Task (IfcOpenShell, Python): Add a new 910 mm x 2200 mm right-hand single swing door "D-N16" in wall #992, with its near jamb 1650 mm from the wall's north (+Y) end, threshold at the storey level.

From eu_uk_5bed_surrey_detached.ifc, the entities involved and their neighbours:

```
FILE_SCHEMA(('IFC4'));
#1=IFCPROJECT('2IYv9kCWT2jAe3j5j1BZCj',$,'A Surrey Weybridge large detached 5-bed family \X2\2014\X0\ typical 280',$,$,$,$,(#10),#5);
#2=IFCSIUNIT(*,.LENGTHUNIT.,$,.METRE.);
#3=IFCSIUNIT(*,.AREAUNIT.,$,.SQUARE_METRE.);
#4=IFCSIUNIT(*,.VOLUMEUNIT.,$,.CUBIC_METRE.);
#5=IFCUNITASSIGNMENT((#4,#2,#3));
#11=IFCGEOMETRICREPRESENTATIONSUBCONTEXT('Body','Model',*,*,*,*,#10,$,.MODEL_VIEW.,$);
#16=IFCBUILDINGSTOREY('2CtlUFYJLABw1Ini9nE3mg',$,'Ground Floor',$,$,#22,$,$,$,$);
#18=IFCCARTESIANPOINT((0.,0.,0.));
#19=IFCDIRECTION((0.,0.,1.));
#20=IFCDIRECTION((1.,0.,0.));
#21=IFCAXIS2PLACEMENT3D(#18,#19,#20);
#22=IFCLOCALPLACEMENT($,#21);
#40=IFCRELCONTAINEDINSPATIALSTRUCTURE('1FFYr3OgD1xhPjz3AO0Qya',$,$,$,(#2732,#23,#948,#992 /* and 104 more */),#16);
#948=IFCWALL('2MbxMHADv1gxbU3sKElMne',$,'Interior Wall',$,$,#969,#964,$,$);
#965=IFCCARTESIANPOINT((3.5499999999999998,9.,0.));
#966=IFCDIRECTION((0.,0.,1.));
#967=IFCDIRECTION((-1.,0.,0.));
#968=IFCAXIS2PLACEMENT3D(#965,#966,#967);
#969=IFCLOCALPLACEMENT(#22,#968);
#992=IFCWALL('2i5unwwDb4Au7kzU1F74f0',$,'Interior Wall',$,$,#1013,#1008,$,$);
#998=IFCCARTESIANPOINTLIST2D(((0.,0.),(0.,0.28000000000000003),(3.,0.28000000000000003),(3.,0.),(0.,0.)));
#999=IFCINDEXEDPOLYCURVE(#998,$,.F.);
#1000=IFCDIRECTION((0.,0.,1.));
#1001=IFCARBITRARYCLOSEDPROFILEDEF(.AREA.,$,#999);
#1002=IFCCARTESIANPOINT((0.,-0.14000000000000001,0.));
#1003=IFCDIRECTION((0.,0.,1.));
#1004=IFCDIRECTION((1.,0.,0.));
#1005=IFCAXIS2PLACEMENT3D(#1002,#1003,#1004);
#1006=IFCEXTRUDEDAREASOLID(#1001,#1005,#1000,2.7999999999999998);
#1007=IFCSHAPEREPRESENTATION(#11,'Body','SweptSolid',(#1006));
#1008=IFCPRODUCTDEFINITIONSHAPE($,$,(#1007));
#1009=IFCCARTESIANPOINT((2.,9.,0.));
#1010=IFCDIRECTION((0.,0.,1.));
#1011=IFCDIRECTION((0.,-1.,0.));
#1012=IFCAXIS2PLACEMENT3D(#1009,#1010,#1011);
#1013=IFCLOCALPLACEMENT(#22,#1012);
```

```python
import numpy as np
import ifcopenshell
import ifcopenshell.api.feature
import ifcopenshell.api.geometry
import ifcopenshell.api.root
import ifcopenshell.api.spatial
import ifcopenshell.geom
import ifcopenshell.util.element
import ifcopenshell.util.placement
import ifcopenshell.util.representation
import ifcopenshell.util.shape
import ifcopenshell.util.unit

model = ifcopenshell.open("eu_uk_5bed_surrey_detached.ifc")
unit_scale = ifcopenshell.util.unit.calculate_unit_scale(model)
settings = ifcopenshell.geom.settings()


def volume(element):
    """Net volume in cubic metres, openings subtracted."""
    shape = ifcopenshell.geom.create_shape(settings, element)
    return ifcopenshell.util.shape.get_volume(shape.geometry)


wall = model.by_guid("2i5unwwDb4Au7kzU1F74f0")
storey = ifcopenshell.util.element.get_container(wall, ifc_class="IfcBuildingStorey")
context = ifcopenshell.util.representation.get_context(model, "Model", "Body", "MODEL_VIEW")
before = volume(wall)

width, height, from_end, sill = 0.91, 2.2, 1.65, 0.0  # metres

# The wall runs along its own X axis, and the end named is its -X end.
wall_shape = ifcopenshell.geom.create_shape(settings, wall)
x, y, z = ifcopenshell.util.shape.get_vertices(wall_shape.geometry).T
start = x.min() + from_end
face, thickness = float(y.min()), float(y.max() - y.min())
wall_matrix = ifcopenshell.util.placement.get_local_placement(wall.ObjectPlacement)
level = ifcopenshell.util.placement.get_local_placement(storey.ObjectPlacement)[2, 3]


def in_wall(x, y):
    """Placement at x, y metres in the wall's axes, at sill height."""
    matrix = wall_matrix.copy()
    matrix[:, 3] = wall_matrix @ np.array([x / unit_scale, y / unit_scale, 0.0, 1.0])
    matrix[2, 3] = level + sill / unit_scale
    return matrix


# Opening: a box that overshoots both wall faces by 50 mm.
opening = ifcopenshell.api.root.create_entity(model, ifc_class="IfcOpeningElement", predefined_type="OPENING")
box = ifcopenshell.api.geometry.add_wall_representation(
    model, context=context, length=width, height=height, thickness=thickness + 0.1
)
ifcopenshell.api.geometry.assign_representation(model, product=opening, representation=box)
ifcopenshell.api.geometry.edit_object_placement(model, product=opening, matrix=in_wall(start, face - 0.05), is_si=False)
ifcopenshell.api.feature.add_feature(model, feature=opening, element=wall)

door = ifcopenshell.api.root.create_entity(model, ifc_class="IfcDoor", name="D-N16", predefined_type="DOOR")
door.OverallWidth, door.OverallHeight = width / unit_scale, height / unit_scale
door.OperationType = "SINGLE_SWING_RIGHT"
body = ifcopenshell.api.geometry.add_door_representation(
    model,
    context=context,
    overall_width=door.OverallWidth,
    overall_height=door.OverallHeight,
    operation_type="SINGLE_SWING_RIGHT",
    lining_properties={"LiningDepth": thickness / unit_scale, "ThresholdDepth": thickness / unit_scale},
)
ifcopenshell.api.geometry.assign_representation(model, product=door, representation=body)
ifcopenshell.api.spatial.assign_container(model, products=[door], relating_structure=storey)
ifcopenshell.api.feature.add_filling(model, opening=opening, element=door)

# The lining spans the wall, so the door starts at the wall face.
ifcopenshell.api.geometry.edit_object_placement(model, product=door, matrix=in_wall(start, face), is_si=False)

after = volume(wall)

print(f"wall volume {before:.3f} -> {after:.3f} m3")

model.write("eu_uk_5bed_surrey_detached_updated.ifc")
```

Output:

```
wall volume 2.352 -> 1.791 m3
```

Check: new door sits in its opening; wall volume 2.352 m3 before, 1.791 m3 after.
